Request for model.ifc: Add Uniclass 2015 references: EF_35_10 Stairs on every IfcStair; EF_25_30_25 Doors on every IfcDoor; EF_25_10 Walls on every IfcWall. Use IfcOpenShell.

First a look at what the model holds.

```python
import ifcopenshell

model = ifcopenshell.open("model.ifc")
print(model.schema)
print("classifications:", [c.Name for c in model.by_type("IfcClassification")])
for ifc_class in ("IfcDoor", "IfcRoof", "IfcStair", "IfcWall", "IfcWindow"):
    print(ifc_class, len(model.by_type(ifc_class)))
```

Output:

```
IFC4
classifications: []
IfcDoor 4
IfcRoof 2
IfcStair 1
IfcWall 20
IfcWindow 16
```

```python
import ifcopenshell
import ifcopenshell.api.classification

model = ifcopenshell.open("model.ifc")

system = ifcopenshell.api.classification.add_classification(model, classification="Uniclass 2015")

codes = {
    "IfcStair": ("EF_35_10", "Stairs"),
    "IfcDoor": ("EF_25_30_25", "Doors"),
    "IfcWall": ("EF_25_10", "Walls"),
}
for ifc_class, (code, name) in codes.items():
    products = model.by_type(ifc_class)
    ifcopenshell.api.classification.add_reference(
        model, products=products, classification=system, identification=code, name=name
    )
    print(code, len(products))

model.write("model_updated.ifc")
```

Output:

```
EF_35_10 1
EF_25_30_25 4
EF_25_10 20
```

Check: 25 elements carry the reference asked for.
